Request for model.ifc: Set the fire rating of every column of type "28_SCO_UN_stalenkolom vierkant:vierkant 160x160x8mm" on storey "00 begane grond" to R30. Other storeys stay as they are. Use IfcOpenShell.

First a look at what the model holds.

```python
import ifcopenshell
import ifcopenshell.util.element

model = ifcopenshell.open("model.ifc")
print(model.schema)
storey = next(s for s in model.by_type("IfcBuildingStorey") if s.Name == "00 begane grond")
columns = [e for e in ifcopenshell.util.element.get_decomposition(storey) if e.is_a("IfcColumn")]
seen = {}
for e in columns:
    element_type = ifcopenshell.util.element.get_type(e)
    key = (element_type.Name if element_type != e and element_type else None, ifcopenshell.util.element.get_pset(e, "Pset_ColumnCommon", "FireRating"))
    seen[key] = seen.get(key, 0) + 1
for (name, value), count in sorted(seen.items(), key=str):
    print(count, "x", name, "|", value)
```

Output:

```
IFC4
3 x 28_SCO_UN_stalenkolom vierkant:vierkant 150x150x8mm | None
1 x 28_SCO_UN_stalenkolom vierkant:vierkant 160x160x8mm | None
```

```python
import ifcopenshell
import ifcopenshell.api.pset
import ifcopenshell.util.element

model = ifcopenshell.open("model.ifc")

storey = next(s for s in model.by_type("IfcBuildingStorey") if s.Name == "00 begane grond")
columns = [e for e in ifcopenshell.util.element.get_decomposition(storey) if e.is_a("IfcColumn")]

count = 0
for e in columns:
    element_type = ifcopenshell.util.element.get_type(e)
    if element_type in (None, e) or element_type.Name != "28_SCO_UN_stalenkolom vierkant:vierkant 160x160x8mm":
        continue
    # add_pset returns the element's existing set when there is one.
    pset = ifcopenshell.api.pset.add_pset(model, product=e, name="Pset_ColumnCommon")
    ifcopenshell.api.pset.edit_pset(model, pset=pset, properties={"FireRating": "R30"})
    count += 1

print(count, "columns updated")

model.write("model_edited.ifc")
```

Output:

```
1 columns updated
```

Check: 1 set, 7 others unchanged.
